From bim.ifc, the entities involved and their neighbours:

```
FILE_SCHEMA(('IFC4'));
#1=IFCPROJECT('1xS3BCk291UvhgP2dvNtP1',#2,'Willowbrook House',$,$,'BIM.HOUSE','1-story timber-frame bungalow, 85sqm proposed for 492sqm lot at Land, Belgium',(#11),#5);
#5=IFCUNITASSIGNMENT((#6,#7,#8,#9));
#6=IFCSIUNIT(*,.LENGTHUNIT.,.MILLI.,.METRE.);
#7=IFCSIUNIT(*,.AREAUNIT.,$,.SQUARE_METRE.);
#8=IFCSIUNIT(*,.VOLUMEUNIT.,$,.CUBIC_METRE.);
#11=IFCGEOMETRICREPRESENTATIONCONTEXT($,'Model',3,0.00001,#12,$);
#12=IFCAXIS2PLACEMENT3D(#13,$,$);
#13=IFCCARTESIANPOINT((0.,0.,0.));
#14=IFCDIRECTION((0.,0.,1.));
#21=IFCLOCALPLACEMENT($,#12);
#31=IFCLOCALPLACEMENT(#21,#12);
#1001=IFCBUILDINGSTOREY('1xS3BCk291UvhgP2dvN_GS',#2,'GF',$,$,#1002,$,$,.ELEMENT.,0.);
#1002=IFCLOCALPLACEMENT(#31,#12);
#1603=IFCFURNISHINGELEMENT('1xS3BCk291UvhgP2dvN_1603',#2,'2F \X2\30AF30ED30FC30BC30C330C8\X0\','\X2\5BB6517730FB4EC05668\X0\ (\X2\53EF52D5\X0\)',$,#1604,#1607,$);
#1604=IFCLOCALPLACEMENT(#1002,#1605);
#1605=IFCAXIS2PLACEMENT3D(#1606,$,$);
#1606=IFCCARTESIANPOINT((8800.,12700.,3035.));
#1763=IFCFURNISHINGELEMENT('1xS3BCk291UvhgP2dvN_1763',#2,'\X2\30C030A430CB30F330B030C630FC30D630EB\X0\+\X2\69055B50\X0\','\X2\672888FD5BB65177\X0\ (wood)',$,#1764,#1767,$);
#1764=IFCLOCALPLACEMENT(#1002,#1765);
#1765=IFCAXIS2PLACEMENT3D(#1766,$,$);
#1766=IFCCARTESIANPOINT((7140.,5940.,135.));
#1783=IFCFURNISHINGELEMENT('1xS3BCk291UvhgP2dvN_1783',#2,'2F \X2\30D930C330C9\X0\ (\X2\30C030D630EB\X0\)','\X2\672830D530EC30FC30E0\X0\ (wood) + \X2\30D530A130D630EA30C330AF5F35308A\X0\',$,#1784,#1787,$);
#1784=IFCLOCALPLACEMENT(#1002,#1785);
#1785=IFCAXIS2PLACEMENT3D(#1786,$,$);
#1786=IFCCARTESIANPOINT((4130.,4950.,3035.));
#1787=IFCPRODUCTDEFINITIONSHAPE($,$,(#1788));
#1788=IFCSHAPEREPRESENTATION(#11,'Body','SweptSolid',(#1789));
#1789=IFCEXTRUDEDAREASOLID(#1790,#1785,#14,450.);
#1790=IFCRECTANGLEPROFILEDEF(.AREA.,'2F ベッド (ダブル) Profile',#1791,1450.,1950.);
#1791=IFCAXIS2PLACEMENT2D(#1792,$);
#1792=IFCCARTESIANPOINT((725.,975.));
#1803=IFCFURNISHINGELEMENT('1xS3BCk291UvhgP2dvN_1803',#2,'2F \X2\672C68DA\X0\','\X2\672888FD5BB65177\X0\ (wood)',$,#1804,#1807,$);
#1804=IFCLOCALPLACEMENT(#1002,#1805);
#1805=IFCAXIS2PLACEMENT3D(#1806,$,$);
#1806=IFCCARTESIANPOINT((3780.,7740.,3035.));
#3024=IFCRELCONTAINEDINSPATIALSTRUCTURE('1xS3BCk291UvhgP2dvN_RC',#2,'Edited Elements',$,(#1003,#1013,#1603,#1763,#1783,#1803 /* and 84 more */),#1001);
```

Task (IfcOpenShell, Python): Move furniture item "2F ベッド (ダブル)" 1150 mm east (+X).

```python
import ifcopenshell
import ifcopenshell.api.geometry
import ifcopenshell.util.placement
import ifcopenshell.util.unit

model = ifcopenshell.open("bim.ifc")
unit_scale = ifcopenshell.util.unit.calculate_unit_scale(model)

item = model.by_guid("1xS3BCk291UvhgP2dvN_1783")
matrix = ifcopenshell.util.placement.get_local_placement(item.ObjectPlacement)
matrix[0, 3] += 1.15 / unit_scale
ifcopenshell.api.geometry.edit_object_placement(model, product=item, matrix=matrix, is_si=False)

print(ifcopenshell.util.placement.get_local_placement(item.ObjectPlacement).round(3) + 0.0)

model.write("bim_edited.ifc")
```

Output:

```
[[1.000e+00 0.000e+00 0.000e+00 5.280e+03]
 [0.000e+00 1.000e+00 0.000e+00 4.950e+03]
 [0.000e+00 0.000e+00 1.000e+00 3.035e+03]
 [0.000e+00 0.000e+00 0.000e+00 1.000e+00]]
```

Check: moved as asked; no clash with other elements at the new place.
